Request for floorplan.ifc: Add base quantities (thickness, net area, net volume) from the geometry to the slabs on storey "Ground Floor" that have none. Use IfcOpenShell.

First a look at what the model holds.

```python
import ifcopenshell
import ifcopenshell.util.element
import ifcopenshell.util.unit

model = ifcopenshell.open("floorplan.ifc")
print(model.schema)
for unit_type in ("LENGTHUNIT", "AREAUNIT", "VOLUMEUNIT"):
    print(unit_type, ifcopenshell.util.unit.calculate_unit_scale(model, unit_type))
storey = next(s for s in model.by_type("IfcBuildingStorey") if s.Name == "Ground Floor")
slabs = [e for e in ifcopenshell.util.element.get_decomposition(storey) if e.is_a("IfcSlab")]
for e in sorted(slabs, key=lambda e: e.id()):
    print(e.id(), e.is_a(), e.Name, list(ifcopenshell.util.element.get_psets(e, qtos_only=True)), sep=" | ")
```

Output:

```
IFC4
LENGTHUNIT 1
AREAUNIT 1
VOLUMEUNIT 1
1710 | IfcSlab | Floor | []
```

```python
import ifcopenshell
import ifcopenshell.api.pset
import ifcopenshell.geom
import ifcopenshell.util.element
import ifcopenshell.util.shape
import ifcopenshell.util.unit

model = ifcopenshell.open("floorplan.ifc")
unit_scale = ifcopenshell.util.unit.calculate_unit_scale(model)
area_scale = ifcopenshell.util.unit.calculate_unit_scale(model, "AREAUNIT")
volume_scale = ifcopenshell.util.unit.calculate_unit_scale(model, "VOLUMEUNIT")
settings = ifcopenshell.geom.settings()

storey = next(s for s in model.by_type("IfcBuildingStorey") if s.Name == "Ground Floor")
slabs = [e for e in ifcopenshell.util.element.get_decomposition(storey) if e.is_a("IfcSlab")]

for e in sorted(slabs, key=lambda e: e.id()):
    if ifcopenshell.util.element.get_psets(e, qtos_only=True, should_inherit=False):
        continue
    # Geometry comes back in metres, in the element's own axes.
    shape = ifcopenshell.geom.create_shape(settings, e)
    values = {
        "Width": ifcopenshell.util.shape.get_z(shape.geometry) / unit_scale,
        "NetArea": ifcopenshell.util.shape.get_footprint_area(shape.geometry) / area_scale,
        "NetVolume": ifcopenshell.util.shape.get_volume(shape.geometry) / volume_scale,
    }
    qto = ifcopenshell.api.pset.add_qto(model, product=e, name="Qto_SlabBaseQuantities")
    ifcopenshell.api.pset.edit_qto(model, qto=qto, properties=values)
    print(e.id(), {k: round(v, 3) for k, v in values.items()})

model.write("floorplan_edited.ifc")
```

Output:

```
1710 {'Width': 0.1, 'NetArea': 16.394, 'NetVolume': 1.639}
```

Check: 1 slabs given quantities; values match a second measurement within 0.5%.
